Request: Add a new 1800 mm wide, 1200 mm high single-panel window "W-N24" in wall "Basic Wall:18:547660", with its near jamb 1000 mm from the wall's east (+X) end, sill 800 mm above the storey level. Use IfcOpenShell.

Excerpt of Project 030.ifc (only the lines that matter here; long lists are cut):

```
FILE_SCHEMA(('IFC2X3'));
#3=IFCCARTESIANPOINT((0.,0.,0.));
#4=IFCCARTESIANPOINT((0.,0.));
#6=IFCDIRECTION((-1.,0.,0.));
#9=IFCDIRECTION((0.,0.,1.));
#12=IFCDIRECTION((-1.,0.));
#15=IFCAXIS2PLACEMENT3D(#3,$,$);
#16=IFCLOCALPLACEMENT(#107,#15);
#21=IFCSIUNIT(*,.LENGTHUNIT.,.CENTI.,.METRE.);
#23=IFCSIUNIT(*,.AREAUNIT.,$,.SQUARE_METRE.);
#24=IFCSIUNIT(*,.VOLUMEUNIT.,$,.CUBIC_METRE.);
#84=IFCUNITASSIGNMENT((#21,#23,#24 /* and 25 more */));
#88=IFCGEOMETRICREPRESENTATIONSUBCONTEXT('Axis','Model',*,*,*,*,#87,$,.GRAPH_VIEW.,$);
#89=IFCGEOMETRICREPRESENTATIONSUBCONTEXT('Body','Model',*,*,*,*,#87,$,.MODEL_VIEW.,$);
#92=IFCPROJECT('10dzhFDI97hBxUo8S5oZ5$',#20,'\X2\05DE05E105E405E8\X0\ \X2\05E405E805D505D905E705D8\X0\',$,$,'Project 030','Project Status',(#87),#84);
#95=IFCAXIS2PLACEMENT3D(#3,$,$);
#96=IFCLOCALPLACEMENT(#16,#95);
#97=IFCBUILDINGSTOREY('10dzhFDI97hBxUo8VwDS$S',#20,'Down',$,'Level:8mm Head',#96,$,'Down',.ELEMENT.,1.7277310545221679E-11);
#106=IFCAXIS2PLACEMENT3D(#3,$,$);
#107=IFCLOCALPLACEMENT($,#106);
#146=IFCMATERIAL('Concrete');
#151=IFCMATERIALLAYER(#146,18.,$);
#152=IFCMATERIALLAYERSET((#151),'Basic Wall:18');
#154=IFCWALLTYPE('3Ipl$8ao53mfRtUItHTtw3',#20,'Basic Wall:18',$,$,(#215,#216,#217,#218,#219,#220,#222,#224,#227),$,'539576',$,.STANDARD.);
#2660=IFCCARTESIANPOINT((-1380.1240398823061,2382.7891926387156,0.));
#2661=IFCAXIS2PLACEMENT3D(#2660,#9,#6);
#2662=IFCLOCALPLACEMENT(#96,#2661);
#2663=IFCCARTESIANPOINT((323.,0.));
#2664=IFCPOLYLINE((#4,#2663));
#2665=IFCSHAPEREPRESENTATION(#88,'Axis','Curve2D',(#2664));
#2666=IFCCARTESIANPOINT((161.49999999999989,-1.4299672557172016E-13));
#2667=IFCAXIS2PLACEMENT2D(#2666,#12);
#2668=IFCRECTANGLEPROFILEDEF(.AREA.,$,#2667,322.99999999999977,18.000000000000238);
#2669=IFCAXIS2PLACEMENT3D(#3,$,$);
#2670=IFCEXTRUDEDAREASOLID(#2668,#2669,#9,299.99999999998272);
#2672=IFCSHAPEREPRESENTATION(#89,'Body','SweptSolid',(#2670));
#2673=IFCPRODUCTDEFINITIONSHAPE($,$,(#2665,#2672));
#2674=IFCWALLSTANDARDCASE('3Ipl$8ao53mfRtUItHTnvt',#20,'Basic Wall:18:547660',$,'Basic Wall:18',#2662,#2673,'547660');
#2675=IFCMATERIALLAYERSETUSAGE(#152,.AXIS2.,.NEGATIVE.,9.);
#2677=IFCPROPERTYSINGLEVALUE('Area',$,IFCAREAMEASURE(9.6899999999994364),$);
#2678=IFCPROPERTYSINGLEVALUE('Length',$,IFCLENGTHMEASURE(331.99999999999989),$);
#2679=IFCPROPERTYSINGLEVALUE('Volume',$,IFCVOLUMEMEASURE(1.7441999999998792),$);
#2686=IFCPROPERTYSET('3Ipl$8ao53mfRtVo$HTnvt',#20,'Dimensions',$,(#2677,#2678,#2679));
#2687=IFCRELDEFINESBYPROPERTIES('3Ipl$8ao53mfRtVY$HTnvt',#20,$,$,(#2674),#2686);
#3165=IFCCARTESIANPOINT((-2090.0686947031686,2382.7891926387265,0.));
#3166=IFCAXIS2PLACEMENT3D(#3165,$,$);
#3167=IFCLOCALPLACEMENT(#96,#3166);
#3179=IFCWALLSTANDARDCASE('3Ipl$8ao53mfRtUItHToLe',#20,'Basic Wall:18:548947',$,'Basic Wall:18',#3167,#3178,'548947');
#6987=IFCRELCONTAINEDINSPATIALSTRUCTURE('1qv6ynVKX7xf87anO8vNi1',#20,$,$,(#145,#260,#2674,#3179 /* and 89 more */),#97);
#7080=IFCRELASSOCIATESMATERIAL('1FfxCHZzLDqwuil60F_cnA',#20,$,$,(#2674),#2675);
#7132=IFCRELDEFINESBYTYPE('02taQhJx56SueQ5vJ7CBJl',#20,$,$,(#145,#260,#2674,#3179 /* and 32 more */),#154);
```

```python
import numpy as np
import ifcopenshell
import ifcopenshell.api.feature
import ifcopenshell.api.geometry
import ifcopenshell.api.pset
import ifcopenshell.api.root
import ifcopenshell.api.spatial
import ifcopenshell.api.type
import ifcopenshell.geom
import ifcopenshell.util.element
import ifcopenshell.util.placement
import ifcopenshell.util.representation
import ifcopenshell.util.shape
import ifcopenshell.util.unit

model = ifcopenshell.open("Project 030.ifc")
unit_scale = ifcopenshell.util.unit.calculate_unit_scale(model)
area_scale = ifcopenshell.util.unit.calculate_unit_scale(model, "AREAUNIT")
volume_scale = ifcopenshell.util.unit.calculate_unit_scale(model, "VOLUMEUNIT")
settings = ifcopenshell.geom.settings()


def volume(element):
    """Net volume in cubic metres, openings subtracted."""
    shape = ifcopenshell.geom.create_shape(settings, element)
    return ifcopenshell.util.shape.get_volume(shape.geometry)


wall = model.by_id(2674)
storey = ifcopenshell.util.element.get_container(wall, ifc_class="IfcBuildingStorey")
context = ifcopenshell.util.representation.get_context(model, "Model", "Body", "MODEL_VIEW")
before = volume(wall)

width, height, from_end, sill = 1.8, 1.2, 1, 0.8  # metres

# The wall runs along its own X axis, and the end named is its -X end.
wall_shape = ifcopenshell.geom.create_shape(settings, wall)
x, y, z = ifcopenshell.util.shape.get_vertices(wall_shape.geometry).T
start = x.min() + from_end
face, thickness = float(y.min()), float(y.max() - y.min())
wall_matrix = ifcopenshell.util.placement.get_local_placement(wall.ObjectPlacement)
level = ifcopenshell.util.placement.get_local_placement(storey.ObjectPlacement)[2, 3]


def in_wall(x, y):
    """Placement at x, y metres in the wall's axes, at sill height."""
    matrix = wall_matrix.copy()
    matrix[:, 3] = wall_matrix @ np.array([x / unit_scale, y / unit_scale, 0.0, 1.0])
    matrix[2, 3] = level + sill / unit_scale
    return matrix


# Opening: a box that overshoots both wall faces by 50 mm.
opening = ifcopenshell.api.root.create_entity(model, ifc_class="IfcOpeningElement")
box = ifcopenshell.api.geometry.add_wall_representation(
    model, context=context, length=width, height=height, thickness=thickness + 0.1
)
ifcopenshell.api.geometry.assign_representation(model, product=opening, representation=box)
ifcopenshell.api.geometry.edit_object_placement(model, product=opening, matrix=in_wall(start, face - 0.05), is_si=False)
ifcopenshell.api.feature.add_feature(model, feature=opening, element=wall)

window = ifcopenshell.api.root.create_entity(model, ifc_class="IfcWindow", name="W-N24")
window.OverallWidth, window.OverallHeight = width / unit_scale, height / unit_scale
body = ifcopenshell.api.geometry.add_window_representation(
    model,
    context=context,
    overall_width=window.OverallWidth,
    overall_height=window.OverallHeight,
    partition_type="SINGLE_PANEL",
)
ifcopenshell.api.geometry.assign_representation(model, product=window, representation=body)
ifcopenshell.api.spatial.assign_container(model, products=[window], relating_structure=storey)
fills = ifcopenshell.api.feature.add_filling(model, opening=opening, element=window)
fills.OwnerHistory = window.OwnerHistory  # required in IFC2X3

# IFC2X3 keeps the operation on the window style.
style = ifcopenshell.api.root.create_entity(model, ifc_class="IfcWindowStyle", name="W-N24")
style.OperationType, style.ConstructionType = "SINGLE_PANEL", "NOTDEFINED"
style.ParameterTakesPrecedence = style.Sizeable = False
ifcopenshell.api.type.assign_type(model, related_objects=[window], relating_type=style)

# Centre the window in the wall's thickness.
ifcopenshell.api.geometry.edit_object_placement(model, product=window, matrix=in_wall(start, face), is_si=False)
window_shape = ifcopenshell.geom.create_shape(settings, window)
depth = ifcopenshell.util.shape.get_vertices(window_shape.geometry)[:, 1]
offset = face + thickness / 2 - (depth.min() + depth.max()) / 2
ifcopenshell.api.geometry.edit_object_placement(model, product=window, matrix=in_wall(start, offset), is_si=False)

after = volume(wall)

# Update the wall's stored quantities.
pset = model.by_id(ifcopenshell.util.element.get_pset(wall, "Dimensions", should_inherit=False)["id"])
ifcopenshell.api.pset.edit_pset(model, pset=pset, properties={
    "Area": model.create_entity("IfcAreaMeasure", after / thickness / area_scale),
    "Volume": model.create_entity("IfcVolumeMeasure", after / volume_scale),
})

print(f"wall volume {before:.3f} -> {after:.3f} m3")

model.write("Project 030_edited.ifc")
```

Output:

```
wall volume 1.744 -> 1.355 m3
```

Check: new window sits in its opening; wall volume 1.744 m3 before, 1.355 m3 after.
